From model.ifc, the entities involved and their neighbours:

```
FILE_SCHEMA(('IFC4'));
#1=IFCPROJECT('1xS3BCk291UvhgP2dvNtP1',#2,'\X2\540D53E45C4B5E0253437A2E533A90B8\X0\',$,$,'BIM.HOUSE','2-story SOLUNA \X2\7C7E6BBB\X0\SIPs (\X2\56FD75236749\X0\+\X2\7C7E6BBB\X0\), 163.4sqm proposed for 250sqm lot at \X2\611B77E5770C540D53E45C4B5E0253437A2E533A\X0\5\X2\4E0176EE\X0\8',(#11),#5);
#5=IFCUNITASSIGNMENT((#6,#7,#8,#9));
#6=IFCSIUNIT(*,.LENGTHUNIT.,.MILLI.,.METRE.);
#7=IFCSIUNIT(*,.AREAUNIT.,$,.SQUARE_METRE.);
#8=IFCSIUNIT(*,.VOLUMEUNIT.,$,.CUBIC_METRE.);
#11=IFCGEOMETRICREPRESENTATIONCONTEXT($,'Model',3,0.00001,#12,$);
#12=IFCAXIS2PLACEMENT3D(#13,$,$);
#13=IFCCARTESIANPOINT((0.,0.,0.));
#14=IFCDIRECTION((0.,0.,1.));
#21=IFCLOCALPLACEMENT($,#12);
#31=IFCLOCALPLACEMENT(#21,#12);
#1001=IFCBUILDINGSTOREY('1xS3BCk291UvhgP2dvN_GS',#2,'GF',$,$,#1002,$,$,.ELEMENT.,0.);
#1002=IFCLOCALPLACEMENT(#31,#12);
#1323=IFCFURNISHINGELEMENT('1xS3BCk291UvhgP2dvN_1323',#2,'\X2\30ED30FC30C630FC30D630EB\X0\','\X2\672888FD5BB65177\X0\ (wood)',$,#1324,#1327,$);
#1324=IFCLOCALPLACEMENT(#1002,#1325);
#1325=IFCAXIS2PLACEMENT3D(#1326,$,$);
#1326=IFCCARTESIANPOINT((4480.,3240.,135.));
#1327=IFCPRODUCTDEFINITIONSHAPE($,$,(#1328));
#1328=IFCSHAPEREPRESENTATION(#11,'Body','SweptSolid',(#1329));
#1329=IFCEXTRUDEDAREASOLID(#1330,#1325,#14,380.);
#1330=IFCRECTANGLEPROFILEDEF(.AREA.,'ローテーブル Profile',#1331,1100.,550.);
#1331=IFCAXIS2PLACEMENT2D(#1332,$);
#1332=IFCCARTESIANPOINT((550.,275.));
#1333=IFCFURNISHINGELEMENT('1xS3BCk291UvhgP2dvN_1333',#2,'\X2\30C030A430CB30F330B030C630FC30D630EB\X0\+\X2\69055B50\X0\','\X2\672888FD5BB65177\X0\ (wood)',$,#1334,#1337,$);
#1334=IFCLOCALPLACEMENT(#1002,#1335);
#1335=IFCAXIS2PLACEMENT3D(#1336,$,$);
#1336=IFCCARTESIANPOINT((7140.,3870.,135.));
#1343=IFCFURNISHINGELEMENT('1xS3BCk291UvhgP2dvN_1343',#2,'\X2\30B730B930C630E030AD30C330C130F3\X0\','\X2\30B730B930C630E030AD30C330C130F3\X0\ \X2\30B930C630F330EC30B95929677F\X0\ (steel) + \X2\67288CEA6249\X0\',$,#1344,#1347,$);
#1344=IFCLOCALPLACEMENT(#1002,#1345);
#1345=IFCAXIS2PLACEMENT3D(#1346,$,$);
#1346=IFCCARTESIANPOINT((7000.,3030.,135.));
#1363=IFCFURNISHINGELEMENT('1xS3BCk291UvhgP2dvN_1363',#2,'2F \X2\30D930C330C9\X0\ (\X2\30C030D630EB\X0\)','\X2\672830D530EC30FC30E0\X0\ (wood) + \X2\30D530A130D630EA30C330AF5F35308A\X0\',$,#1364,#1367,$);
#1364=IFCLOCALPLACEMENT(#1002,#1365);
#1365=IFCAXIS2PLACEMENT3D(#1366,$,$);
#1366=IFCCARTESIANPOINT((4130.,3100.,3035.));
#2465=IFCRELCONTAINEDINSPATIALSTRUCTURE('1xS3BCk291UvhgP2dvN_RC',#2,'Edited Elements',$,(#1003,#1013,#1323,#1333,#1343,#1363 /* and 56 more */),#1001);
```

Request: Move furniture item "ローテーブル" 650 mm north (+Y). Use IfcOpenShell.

```python
import ifcopenshell
import ifcopenshell.api.geometry
import ifcopenshell.util.placement
import ifcopenshell.util.unit

model = ifcopenshell.open("model.ifc")
unit_scale = ifcopenshell.util.unit.calculate_unit_scale(model)

item = model.by_guid("1xS3BCk291UvhgP2dvN_1323")
matrix = ifcopenshell.util.placement.get_local_placement(item.ObjectPlacement)
matrix[1, 3] += 0.65 / unit_scale
ifcopenshell.api.geometry.edit_object_placement(model, product=item, matrix=matrix, is_si=False)

print(ifcopenshell.util.placement.get_local_placement(item.ObjectPlacement).round(3) + 0.0)

model.write("model_v2.ifc")
```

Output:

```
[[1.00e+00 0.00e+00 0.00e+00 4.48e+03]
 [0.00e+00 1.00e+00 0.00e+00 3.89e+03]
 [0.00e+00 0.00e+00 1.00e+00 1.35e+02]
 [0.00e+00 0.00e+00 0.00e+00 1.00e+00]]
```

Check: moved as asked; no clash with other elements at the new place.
